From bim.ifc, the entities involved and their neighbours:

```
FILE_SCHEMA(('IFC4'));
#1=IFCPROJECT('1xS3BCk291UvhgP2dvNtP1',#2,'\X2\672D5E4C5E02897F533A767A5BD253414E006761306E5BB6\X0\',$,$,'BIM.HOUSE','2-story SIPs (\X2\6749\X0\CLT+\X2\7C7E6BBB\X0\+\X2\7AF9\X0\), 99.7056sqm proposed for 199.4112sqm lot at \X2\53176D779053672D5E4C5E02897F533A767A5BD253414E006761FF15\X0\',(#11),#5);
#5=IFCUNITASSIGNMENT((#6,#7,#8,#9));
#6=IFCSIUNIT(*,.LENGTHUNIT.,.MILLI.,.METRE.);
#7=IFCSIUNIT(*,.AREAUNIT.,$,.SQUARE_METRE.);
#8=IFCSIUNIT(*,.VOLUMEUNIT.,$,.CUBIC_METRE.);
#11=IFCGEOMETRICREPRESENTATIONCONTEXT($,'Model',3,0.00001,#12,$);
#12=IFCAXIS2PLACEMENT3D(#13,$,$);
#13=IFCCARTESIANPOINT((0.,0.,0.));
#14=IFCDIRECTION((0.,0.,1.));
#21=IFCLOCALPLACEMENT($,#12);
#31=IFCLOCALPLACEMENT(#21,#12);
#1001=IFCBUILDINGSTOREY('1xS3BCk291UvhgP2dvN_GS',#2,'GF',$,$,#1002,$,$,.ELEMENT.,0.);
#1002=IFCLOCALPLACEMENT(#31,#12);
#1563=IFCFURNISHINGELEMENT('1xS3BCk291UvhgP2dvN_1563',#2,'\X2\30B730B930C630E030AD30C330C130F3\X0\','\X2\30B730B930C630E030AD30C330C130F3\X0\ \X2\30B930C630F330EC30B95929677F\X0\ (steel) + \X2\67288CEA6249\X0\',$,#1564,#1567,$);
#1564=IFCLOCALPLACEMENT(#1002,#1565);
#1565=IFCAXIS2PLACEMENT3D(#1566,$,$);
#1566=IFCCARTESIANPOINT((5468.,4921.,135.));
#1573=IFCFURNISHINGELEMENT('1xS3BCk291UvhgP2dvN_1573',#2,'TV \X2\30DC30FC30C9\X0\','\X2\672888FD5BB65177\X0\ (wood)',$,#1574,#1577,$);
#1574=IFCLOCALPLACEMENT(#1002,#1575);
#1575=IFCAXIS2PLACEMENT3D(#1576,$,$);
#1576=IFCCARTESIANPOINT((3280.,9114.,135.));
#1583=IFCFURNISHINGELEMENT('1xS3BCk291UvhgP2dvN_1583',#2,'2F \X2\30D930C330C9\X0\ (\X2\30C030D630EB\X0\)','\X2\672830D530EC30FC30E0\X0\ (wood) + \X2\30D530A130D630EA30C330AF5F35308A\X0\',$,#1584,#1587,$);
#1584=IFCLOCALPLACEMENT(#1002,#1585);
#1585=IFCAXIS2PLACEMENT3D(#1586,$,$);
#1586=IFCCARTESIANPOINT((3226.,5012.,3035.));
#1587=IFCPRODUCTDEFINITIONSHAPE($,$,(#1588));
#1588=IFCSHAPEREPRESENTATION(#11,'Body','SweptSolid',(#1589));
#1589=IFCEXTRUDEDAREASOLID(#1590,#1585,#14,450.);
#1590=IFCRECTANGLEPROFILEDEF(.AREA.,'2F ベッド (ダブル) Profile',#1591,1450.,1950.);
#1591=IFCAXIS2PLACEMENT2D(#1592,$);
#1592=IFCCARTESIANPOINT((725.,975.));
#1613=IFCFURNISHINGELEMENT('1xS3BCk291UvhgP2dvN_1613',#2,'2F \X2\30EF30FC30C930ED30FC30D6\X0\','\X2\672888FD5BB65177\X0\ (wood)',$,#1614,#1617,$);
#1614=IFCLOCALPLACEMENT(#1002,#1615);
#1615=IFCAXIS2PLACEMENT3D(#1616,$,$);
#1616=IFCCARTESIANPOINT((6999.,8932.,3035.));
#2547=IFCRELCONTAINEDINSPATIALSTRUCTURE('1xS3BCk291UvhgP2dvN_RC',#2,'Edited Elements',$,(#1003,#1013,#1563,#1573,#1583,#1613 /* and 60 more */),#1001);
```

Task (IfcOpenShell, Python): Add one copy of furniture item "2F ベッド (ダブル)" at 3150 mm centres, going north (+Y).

```python
import numpy as np
import ifcopenshell
import ifcopenshell.api.geometry
import ifcopenshell.api.root
import ifcopenshell.util.element
import ifcopenshell.util.placement
import ifcopenshell.util.unit

model = ifcopenshell.open("bim.ifc")
unit_scale = ifcopenshell.util.unit.calculate_unit_scale(model)


def reuse_history(source, copy):
    """copy_class also copies each property set's owner history, people and application; keep the originals."""
    for rel in copy.IsDefinedBy:
        if rel.is_a("IfcRelDefinesByProperties") and (history := rel.RelatingPropertyDefinition.OwnerHistory):
            rel.RelatingPropertyDefinition.OwnerHistory = source.OwnerHistory
            ifcopenshell.util.element.remove_deep2(model, history)


source = model.by_id(1583)
base = ifcopenshell.util.placement.get_local_placement(source.ObjectPlacement)
step = np.array([0.0, 1.0, 0.0]) * 3.15 / unit_scale

for i in range(1, 2):
    copy = ifcopenshell.api.root.copy_class(model, product=source)
    copy.Representation = ifcopenshell.util.element.copy_deep(
        model, source.Representation, exclude=["IfcGeometricRepresentationContext", "IfcRepresentationMap"]
    )
    reuse_history(source, copy)
    matrix = base.copy()
    matrix[:3, 3] += i * step
    print("added at", matrix[:3, 3].round(3) + 0.0)
    ifcopenshell.api.geometry.edit_object_placement(model, product=copy, matrix=matrix, is_si=False)

model.write("bim_v2.ifc")
```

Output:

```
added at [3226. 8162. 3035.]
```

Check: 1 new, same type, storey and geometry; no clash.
